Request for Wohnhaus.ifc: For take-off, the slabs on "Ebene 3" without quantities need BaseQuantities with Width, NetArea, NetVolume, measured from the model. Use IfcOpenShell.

First a look at what the model holds.

```python
import ifcopenshell
import ifcopenshell.util.element
import ifcopenshell.util.unit

model = ifcopenshell.open("Wohnhaus.ifc")
print(model.schema)
for unit_type in ("LENGTHUNIT", "AREAUNIT", "VOLUMEUNIT"):
    print(unit_type, ifcopenshell.util.unit.calculate_unit_scale(model, unit_type))
storey = next(s for s in model.by_type("IfcBuildingStorey") if s.Name == "Ebene 3")
slabs = [e for e in ifcopenshell.util.element.get_decomposition(storey) if e.is_a("IfcSlab")]
for e in sorted(slabs, key=lambda e: e.id()):
    print(e.id(), e.is_a(), e.Name, list(ifcopenshell.util.element.get_psets(e, qtos_only=True)), sep=" | ")
```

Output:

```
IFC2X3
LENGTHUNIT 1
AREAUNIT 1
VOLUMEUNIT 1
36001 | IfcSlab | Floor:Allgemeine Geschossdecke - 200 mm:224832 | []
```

```python
import ifcopenshell
import ifcopenshell.api.pset
import ifcopenshell.geom
import ifcopenshell.util.element
import ifcopenshell.util.shape
import ifcopenshell.util.unit

model = ifcopenshell.open("Wohnhaus.ifc")
unit_scale = ifcopenshell.util.unit.calculate_unit_scale(model)
area_scale = ifcopenshell.util.unit.calculate_unit_scale(model, "AREAUNIT")
volume_scale = ifcopenshell.util.unit.calculate_unit_scale(model, "VOLUMEUNIT")
settings = ifcopenshell.geom.settings()

storey = next(s for s in model.by_type("IfcBuildingStorey") if s.Name == "Ebene 3")
slabs = [e for e in ifcopenshell.util.element.get_decomposition(storey) if e.is_a("IfcSlab")]

for e in sorted(slabs, key=lambda e: e.id()):
    if ifcopenshell.util.element.get_psets(e, qtos_only=True, should_inherit=False):
        continue
    # Geometry comes back in metres, in the element's own axes.
    shape = ifcopenshell.geom.create_shape(settings, e)
    values = {
        "Width": ifcopenshell.util.shape.get_z(shape.geometry) / unit_scale,
        "NetArea": ifcopenshell.util.shape.get_footprint_area(shape.geometry) / area_scale,
        "NetVolume": ifcopenshell.util.shape.get_volume(shape.geometry) / volume_scale,
    }
    qto = ifcopenshell.api.pset.add_qto(model, product=e, name="BaseQuantities")
    ifcopenshell.api.pset.edit_qto(model, qto=qto, properties=values)
    print(e.id(), {k: round(v, 3) for k, v in values.items()})

model.write("Wohnhaus_updated.ifc")
```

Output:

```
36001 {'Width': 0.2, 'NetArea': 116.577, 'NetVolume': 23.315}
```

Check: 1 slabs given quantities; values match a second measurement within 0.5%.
